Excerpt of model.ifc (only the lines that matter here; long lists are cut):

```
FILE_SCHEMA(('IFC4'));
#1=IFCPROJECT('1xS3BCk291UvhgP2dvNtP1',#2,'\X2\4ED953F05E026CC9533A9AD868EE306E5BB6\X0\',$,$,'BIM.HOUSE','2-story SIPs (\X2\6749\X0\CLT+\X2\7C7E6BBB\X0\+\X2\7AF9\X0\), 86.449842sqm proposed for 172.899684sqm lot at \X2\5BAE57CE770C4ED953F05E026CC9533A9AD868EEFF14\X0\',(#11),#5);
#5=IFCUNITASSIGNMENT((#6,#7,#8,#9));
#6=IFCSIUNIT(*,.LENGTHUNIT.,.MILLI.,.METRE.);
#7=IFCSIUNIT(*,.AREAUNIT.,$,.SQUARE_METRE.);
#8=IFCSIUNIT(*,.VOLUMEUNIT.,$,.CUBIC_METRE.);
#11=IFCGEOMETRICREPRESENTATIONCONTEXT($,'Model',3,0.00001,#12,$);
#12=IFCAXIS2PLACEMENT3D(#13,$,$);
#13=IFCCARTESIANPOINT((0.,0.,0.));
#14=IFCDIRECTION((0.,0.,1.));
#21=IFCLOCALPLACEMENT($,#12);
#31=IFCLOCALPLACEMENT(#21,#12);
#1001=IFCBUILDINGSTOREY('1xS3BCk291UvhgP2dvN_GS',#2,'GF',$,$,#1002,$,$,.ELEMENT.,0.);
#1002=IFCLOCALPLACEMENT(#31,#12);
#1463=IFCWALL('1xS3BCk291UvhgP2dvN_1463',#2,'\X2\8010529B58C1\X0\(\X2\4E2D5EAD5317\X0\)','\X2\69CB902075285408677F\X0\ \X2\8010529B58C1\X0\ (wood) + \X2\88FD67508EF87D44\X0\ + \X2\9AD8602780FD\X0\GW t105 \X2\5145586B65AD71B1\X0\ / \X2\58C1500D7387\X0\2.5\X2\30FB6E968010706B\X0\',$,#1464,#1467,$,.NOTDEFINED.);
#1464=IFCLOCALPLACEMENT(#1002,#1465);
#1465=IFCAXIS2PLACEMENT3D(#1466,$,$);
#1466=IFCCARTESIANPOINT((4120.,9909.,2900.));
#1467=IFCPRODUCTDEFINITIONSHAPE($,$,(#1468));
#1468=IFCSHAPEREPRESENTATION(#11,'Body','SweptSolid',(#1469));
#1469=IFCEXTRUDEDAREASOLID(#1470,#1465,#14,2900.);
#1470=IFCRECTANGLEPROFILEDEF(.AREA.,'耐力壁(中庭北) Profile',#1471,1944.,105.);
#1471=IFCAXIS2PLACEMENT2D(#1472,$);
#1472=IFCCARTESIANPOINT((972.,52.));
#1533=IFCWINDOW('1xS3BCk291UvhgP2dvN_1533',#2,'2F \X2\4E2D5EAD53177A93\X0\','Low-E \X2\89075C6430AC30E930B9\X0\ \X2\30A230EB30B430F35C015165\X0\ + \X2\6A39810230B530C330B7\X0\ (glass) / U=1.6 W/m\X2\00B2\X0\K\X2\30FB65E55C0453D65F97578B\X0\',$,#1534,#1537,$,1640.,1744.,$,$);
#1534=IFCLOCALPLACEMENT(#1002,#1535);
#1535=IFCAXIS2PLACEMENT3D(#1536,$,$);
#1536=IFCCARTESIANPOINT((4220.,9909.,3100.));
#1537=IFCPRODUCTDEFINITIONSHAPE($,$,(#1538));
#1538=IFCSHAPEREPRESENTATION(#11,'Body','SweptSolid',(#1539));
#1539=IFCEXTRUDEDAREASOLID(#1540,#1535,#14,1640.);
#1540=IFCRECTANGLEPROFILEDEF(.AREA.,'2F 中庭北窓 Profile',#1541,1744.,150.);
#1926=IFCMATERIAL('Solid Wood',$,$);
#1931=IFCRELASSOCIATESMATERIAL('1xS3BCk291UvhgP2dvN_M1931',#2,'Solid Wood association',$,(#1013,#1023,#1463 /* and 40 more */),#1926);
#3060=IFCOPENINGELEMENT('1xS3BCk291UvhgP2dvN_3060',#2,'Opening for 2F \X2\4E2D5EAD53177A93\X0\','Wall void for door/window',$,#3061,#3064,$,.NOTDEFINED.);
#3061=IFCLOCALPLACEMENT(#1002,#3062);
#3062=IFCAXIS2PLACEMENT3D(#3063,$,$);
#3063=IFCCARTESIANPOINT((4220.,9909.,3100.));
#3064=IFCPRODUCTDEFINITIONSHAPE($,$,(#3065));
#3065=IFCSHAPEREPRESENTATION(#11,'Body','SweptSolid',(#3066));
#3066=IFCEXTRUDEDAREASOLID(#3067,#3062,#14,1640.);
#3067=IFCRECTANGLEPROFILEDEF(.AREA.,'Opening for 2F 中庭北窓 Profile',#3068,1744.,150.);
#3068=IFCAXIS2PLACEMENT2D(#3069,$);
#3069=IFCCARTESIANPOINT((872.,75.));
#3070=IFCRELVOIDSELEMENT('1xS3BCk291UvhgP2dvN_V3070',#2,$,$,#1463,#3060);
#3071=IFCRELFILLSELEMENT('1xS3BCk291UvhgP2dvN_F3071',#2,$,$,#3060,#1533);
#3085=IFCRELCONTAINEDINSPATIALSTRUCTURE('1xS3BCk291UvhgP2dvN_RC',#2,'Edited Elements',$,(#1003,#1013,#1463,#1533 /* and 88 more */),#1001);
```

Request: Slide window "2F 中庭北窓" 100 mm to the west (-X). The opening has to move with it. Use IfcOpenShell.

```python
import ifcopenshell
import ifcopenshell.api.geometry
import ifcopenshell.util.placement
import ifcopenshell.util.unit

model = ifcopenshell.open("model.ifc")
unit_scale = ifcopenshell.util.unit.calculate_unit_scale(model)

window = model.by_guid("1xS3BCk291UvhgP2dvN_1533")
opening = window.FillsVoids[0].RelatingOpeningElement
wall = opening.VoidsElements[0].RelatingBuildingElement

wall_matrix = ifcopenshell.util.placement.get_local_placement(wall.ObjectPlacement)
shift = wall_matrix[:3, 0] * -0.1 / unit_scale
before = ifcopenshell.util.placement.get_local_placement(window.ObjectPlacement)[:3, 3].copy()

# The window is not placed relative to its opening, so move both.
for product in (opening, window):
    matrix = ifcopenshell.util.placement.get_local_placement(product.ObjectPlacement)
    matrix[:3, 3] += shift
    ifcopenshell.api.geometry.edit_object_placement(model, product=product, matrix=matrix, is_si=False)

after = ifcopenshell.util.placement.get_local_placement(window.ObjectPlacement)[:3, 3]
print("window moved by", (after - before).round(3) + 0.0)

model.write("model_rev.ifc")
```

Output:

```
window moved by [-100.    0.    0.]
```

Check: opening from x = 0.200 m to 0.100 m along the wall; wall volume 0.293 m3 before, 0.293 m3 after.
